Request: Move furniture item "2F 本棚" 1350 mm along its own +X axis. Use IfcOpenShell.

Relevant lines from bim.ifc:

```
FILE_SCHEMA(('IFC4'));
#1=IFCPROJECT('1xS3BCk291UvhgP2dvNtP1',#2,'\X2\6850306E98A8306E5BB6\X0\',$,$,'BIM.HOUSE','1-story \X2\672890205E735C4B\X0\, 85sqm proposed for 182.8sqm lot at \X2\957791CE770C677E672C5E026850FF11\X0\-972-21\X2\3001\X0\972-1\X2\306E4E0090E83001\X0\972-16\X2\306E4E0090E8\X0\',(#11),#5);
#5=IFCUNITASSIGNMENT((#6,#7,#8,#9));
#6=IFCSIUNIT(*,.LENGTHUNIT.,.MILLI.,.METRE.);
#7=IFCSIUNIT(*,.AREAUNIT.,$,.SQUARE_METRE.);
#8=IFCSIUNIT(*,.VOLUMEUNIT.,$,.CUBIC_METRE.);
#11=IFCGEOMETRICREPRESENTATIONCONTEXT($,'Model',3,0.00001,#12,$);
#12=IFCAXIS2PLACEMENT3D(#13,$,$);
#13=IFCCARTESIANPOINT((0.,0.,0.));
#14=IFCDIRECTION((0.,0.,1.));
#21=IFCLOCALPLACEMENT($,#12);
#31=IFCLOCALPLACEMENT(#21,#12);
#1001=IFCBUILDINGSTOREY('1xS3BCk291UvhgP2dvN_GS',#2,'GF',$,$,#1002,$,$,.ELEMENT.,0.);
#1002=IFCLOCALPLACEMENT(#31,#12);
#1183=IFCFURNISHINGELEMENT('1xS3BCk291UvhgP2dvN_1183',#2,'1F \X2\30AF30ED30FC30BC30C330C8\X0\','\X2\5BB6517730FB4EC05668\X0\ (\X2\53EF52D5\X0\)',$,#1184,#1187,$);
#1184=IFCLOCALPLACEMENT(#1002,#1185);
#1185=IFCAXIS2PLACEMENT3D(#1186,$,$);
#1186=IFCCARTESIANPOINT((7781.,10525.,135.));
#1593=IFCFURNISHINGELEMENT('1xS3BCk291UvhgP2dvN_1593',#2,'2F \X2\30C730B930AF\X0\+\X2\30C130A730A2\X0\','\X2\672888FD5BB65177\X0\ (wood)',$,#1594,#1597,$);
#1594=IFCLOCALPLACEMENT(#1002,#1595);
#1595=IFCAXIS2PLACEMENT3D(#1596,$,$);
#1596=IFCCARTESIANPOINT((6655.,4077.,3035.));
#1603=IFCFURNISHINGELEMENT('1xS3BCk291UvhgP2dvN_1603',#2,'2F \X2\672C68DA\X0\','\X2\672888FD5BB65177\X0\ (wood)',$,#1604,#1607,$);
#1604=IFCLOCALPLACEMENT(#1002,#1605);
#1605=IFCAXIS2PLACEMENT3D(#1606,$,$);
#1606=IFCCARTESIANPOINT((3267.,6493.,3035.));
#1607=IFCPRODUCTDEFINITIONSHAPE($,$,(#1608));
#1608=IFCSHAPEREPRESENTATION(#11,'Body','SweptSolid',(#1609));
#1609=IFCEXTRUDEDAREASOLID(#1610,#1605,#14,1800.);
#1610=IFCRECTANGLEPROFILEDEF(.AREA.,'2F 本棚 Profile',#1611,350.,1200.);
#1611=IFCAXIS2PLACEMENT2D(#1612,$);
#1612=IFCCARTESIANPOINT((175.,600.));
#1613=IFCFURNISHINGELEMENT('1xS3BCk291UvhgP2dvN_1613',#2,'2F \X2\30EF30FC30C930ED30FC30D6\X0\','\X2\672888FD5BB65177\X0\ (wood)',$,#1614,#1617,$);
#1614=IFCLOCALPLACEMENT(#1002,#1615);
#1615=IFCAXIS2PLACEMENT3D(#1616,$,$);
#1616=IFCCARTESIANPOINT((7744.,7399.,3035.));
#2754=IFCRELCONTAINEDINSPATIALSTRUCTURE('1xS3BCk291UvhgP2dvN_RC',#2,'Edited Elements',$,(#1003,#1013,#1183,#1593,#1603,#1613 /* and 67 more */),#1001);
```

```python
import ifcopenshell
import ifcopenshell.api.geometry
import ifcopenshell.util.placement

model = ifcopenshell.open("bim.ifc")

item = model.by_guid("1xS3BCk291UvhgP2dvN_1603")
matrix = ifcopenshell.util.placement.get_local_placement(item.ObjectPlacement)
matrix[:3, 3] += matrix[:3, 0] * 1350.0
ifcopenshell.api.geometry.edit_object_placement(model, product=item, matrix=matrix, is_si=False)

print(ifcopenshell.util.placement.get_local_placement(item.ObjectPlacement).round(3) + 0.0)

model.write("bim_v2.ifc")
```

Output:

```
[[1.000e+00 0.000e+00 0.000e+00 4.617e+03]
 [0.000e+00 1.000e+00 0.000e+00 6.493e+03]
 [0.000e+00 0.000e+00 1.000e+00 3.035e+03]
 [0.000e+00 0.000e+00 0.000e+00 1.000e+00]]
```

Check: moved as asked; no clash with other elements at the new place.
